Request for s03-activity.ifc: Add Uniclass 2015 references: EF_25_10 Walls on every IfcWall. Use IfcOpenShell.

First a look at what the model holds.

```python
import ifcopenshell

model = ifcopenshell.open("s03-activity.ifc")
print(model.schema)
print("classifications:", [c.Name for c in model.by_type("IfcClassification")])
for ifc_class in ("IfcDoor", "IfcRoof", "IfcStair", "IfcWall", "IfcWindow"):
    print(ifc_class, len(model.by_type(ifc_class)))
```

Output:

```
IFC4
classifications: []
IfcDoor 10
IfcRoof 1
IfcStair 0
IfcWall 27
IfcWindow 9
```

```python
import ifcopenshell
import ifcopenshell.api.classification

model = ifcopenshell.open("s03-activity.ifc")

system = ifcopenshell.api.classification.add_classification(model, classification="Uniclass 2015")

codes = {
    "IfcWall": ("EF_25_10", "Walls"),
}
for ifc_class, (code, name) in codes.items():
    products = model.by_type(ifc_class)
    ifcopenshell.api.classification.add_reference(
        model, products=products, classification=system, identification=code, name=name
    )
    print(code, len(products))

model.write("s03-activity_updated.ifc")
```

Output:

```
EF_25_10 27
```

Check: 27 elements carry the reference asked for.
